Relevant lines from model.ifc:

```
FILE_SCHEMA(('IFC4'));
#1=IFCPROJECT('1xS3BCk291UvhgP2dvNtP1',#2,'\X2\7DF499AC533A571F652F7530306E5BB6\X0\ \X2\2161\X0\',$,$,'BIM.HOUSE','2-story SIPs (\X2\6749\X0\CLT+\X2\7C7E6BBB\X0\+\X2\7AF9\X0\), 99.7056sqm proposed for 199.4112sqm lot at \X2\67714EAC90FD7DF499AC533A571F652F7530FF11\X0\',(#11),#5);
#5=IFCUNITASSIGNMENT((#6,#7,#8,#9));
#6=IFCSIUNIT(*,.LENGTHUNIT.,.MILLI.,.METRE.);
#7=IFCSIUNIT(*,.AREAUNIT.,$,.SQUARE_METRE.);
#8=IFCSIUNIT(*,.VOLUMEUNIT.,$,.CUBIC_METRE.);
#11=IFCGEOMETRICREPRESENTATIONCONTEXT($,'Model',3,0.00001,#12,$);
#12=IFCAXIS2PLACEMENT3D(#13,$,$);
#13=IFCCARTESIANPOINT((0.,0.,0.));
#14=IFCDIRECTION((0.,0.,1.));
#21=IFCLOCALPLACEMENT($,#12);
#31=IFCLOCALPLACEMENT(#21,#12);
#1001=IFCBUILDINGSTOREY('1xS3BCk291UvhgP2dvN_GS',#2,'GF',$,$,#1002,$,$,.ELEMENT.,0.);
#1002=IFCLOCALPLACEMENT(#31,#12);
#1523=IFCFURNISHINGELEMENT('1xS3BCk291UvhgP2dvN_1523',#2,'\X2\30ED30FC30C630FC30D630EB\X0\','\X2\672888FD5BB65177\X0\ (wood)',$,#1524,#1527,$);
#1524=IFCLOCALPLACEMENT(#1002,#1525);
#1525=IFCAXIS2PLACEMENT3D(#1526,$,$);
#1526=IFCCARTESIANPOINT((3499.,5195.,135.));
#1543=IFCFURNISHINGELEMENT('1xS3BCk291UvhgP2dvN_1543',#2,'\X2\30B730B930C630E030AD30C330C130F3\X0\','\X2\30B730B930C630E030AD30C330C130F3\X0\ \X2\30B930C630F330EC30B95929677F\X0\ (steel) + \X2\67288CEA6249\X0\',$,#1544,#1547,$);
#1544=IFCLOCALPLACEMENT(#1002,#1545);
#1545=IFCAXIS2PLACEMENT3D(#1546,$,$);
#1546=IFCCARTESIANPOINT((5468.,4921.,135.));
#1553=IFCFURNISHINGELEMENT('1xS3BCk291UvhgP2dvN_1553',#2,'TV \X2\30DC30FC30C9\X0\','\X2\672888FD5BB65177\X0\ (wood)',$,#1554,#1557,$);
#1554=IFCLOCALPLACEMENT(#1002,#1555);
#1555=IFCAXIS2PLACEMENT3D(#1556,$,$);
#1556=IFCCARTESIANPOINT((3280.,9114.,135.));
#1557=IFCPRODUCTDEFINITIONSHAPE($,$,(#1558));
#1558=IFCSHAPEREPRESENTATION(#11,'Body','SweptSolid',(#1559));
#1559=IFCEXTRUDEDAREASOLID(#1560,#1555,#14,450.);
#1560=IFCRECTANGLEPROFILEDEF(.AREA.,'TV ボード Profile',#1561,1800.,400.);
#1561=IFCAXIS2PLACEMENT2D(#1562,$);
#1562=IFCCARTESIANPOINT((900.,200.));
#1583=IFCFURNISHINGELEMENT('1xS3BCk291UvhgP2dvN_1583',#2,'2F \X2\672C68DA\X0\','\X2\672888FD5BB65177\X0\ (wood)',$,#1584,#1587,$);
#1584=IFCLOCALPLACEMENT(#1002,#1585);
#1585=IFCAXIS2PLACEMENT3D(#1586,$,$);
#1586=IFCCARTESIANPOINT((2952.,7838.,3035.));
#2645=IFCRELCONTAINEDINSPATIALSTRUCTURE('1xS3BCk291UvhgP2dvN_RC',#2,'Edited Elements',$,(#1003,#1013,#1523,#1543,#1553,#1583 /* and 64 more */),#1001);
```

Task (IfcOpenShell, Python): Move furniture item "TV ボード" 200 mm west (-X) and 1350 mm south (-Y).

```python
import ifcopenshell
import ifcopenshell.api.geometry
import ifcopenshell.util.placement

model = ifcopenshell.open("model.ifc")

item = model.by_id(1553)
matrix = ifcopenshell.util.placement.get_local_placement(item.ObjectPlacement)
matrix[0, 3] -= 200.0
matrix[1, 3] -= 1350.0
ifcopenshell.api.geometry.edit_object_placement(model, product=item, matrix=matrix, is_si=False)

print(ifcopenshell.util.placement.get_local_placement(item.ObjectPlacement).round(3) + 0.0)

model.write("model_rev.ifc")
```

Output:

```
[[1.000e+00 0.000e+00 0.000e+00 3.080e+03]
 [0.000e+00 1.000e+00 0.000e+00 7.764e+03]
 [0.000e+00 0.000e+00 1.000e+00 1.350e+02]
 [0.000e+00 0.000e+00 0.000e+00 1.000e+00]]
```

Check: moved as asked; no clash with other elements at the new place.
